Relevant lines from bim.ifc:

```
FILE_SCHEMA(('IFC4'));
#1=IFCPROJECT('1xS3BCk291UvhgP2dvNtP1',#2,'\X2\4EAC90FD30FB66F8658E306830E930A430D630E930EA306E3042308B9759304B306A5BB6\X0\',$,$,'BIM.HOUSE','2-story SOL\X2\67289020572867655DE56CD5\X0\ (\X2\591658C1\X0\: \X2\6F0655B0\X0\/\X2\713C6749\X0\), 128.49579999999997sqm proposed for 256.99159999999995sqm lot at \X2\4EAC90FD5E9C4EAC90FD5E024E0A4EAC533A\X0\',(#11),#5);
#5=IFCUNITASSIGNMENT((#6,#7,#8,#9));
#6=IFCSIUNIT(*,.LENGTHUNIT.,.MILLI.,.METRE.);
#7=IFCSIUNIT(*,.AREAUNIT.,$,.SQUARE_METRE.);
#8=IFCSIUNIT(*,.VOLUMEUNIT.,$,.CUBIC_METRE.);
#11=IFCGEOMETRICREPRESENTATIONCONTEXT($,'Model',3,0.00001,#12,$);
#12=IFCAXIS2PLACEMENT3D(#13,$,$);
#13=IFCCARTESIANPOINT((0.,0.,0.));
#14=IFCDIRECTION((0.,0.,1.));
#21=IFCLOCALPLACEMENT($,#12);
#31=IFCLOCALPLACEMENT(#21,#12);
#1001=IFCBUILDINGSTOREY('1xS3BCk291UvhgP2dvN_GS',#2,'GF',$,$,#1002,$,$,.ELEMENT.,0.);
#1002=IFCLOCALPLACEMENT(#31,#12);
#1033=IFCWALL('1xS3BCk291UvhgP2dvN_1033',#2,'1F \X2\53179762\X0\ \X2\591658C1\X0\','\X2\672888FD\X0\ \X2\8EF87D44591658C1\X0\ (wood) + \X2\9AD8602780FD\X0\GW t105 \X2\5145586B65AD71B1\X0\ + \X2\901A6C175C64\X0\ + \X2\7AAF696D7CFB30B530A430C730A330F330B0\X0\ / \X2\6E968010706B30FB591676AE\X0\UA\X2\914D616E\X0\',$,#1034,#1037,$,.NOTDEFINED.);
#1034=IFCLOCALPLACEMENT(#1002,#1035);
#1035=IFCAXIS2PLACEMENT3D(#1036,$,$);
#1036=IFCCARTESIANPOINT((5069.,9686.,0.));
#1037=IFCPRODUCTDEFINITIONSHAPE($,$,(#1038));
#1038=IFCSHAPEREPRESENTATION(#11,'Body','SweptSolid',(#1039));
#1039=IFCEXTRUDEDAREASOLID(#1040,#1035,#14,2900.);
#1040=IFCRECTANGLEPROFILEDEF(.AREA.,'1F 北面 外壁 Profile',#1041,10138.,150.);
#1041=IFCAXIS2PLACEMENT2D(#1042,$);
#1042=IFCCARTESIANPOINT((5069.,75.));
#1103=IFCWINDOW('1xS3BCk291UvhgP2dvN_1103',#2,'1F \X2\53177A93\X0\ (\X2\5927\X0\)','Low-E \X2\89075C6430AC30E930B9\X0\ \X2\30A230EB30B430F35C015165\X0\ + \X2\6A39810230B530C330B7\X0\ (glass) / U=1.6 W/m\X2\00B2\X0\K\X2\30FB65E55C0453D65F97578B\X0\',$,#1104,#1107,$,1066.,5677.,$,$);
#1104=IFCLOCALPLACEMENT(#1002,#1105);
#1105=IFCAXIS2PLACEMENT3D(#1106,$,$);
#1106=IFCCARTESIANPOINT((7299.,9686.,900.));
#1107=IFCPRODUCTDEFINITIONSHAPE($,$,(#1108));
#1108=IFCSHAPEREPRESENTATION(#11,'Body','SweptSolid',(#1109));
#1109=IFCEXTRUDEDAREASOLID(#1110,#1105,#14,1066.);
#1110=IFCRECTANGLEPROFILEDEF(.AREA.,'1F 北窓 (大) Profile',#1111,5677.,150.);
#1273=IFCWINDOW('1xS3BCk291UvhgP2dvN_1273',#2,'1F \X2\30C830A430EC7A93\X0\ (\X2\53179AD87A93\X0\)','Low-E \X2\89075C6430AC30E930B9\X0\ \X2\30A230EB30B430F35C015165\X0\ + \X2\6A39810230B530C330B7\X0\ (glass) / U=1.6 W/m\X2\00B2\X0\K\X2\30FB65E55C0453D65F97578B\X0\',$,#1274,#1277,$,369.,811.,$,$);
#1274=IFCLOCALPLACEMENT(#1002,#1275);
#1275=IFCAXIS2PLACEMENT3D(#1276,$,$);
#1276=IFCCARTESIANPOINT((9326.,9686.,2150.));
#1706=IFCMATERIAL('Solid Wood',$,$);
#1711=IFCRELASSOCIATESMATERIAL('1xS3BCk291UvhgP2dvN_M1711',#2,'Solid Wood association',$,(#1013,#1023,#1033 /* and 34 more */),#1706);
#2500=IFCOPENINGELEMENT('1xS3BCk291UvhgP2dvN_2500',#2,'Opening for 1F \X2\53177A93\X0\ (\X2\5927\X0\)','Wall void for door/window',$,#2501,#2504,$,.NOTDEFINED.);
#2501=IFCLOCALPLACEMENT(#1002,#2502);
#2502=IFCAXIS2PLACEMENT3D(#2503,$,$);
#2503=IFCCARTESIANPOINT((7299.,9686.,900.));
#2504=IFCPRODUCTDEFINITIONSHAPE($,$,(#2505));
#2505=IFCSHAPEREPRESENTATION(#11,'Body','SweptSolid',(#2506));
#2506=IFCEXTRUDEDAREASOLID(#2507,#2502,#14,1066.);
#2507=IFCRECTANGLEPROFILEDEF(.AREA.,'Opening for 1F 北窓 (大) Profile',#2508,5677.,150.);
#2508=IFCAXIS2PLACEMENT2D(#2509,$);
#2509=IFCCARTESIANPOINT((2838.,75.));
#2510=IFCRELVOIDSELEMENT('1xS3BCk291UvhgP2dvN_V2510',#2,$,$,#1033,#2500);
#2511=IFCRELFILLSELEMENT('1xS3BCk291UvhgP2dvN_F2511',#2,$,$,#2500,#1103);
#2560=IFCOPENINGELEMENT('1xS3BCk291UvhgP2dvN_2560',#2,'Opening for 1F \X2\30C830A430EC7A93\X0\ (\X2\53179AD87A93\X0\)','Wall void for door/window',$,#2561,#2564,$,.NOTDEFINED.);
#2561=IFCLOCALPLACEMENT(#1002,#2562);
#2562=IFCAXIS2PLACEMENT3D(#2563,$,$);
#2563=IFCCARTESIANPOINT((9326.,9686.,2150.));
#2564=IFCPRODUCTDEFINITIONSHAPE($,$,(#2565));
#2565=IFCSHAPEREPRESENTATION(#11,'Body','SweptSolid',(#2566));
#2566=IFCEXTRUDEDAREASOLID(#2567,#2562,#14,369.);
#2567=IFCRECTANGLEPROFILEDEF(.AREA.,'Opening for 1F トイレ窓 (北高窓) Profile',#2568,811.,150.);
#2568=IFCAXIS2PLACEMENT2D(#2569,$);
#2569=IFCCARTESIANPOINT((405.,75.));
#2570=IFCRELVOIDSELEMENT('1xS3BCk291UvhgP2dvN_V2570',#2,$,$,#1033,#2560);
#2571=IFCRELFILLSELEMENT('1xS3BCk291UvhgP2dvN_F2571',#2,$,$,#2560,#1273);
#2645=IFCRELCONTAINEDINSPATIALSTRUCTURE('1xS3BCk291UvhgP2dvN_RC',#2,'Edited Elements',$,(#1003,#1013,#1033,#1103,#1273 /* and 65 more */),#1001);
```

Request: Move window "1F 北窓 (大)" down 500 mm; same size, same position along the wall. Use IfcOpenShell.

```python
import numpy as np
import ifcopenshell
import ifcopenshell.api.geometry
import ifcopenshell.util.placement
import ifcopenshell.util.unit

model = ifcopenshell.open("bim.ifc")
unit_scale = ifcopenshell.util.unit.calculate_unit_scale(model)

window = model.by_guid("1xS3BCk291UvhgP2dvN_1103")
opening = window.FillsVoids[0].RelatingOpeningElement
dz = -0.5 / unit_scale

shift = np.array([0.0, 0.0, dz])
# The window is not placed relative to its opening, so move both.
for product in (opening, window):
    matrix = ifcopenshell.util.placement.get_local_placement(product.ObjectPlacement)
    matrix[:3, 3] += shift
    ifcopenshell.api.geometry.edit_object_placement(model, product=product, matrix=matrix, is_si=False)

print(f"moved by {dz * unit_scale:+.3f} m")

model.write("bim_v2.ifc")
```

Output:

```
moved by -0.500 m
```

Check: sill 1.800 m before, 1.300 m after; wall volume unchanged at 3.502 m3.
